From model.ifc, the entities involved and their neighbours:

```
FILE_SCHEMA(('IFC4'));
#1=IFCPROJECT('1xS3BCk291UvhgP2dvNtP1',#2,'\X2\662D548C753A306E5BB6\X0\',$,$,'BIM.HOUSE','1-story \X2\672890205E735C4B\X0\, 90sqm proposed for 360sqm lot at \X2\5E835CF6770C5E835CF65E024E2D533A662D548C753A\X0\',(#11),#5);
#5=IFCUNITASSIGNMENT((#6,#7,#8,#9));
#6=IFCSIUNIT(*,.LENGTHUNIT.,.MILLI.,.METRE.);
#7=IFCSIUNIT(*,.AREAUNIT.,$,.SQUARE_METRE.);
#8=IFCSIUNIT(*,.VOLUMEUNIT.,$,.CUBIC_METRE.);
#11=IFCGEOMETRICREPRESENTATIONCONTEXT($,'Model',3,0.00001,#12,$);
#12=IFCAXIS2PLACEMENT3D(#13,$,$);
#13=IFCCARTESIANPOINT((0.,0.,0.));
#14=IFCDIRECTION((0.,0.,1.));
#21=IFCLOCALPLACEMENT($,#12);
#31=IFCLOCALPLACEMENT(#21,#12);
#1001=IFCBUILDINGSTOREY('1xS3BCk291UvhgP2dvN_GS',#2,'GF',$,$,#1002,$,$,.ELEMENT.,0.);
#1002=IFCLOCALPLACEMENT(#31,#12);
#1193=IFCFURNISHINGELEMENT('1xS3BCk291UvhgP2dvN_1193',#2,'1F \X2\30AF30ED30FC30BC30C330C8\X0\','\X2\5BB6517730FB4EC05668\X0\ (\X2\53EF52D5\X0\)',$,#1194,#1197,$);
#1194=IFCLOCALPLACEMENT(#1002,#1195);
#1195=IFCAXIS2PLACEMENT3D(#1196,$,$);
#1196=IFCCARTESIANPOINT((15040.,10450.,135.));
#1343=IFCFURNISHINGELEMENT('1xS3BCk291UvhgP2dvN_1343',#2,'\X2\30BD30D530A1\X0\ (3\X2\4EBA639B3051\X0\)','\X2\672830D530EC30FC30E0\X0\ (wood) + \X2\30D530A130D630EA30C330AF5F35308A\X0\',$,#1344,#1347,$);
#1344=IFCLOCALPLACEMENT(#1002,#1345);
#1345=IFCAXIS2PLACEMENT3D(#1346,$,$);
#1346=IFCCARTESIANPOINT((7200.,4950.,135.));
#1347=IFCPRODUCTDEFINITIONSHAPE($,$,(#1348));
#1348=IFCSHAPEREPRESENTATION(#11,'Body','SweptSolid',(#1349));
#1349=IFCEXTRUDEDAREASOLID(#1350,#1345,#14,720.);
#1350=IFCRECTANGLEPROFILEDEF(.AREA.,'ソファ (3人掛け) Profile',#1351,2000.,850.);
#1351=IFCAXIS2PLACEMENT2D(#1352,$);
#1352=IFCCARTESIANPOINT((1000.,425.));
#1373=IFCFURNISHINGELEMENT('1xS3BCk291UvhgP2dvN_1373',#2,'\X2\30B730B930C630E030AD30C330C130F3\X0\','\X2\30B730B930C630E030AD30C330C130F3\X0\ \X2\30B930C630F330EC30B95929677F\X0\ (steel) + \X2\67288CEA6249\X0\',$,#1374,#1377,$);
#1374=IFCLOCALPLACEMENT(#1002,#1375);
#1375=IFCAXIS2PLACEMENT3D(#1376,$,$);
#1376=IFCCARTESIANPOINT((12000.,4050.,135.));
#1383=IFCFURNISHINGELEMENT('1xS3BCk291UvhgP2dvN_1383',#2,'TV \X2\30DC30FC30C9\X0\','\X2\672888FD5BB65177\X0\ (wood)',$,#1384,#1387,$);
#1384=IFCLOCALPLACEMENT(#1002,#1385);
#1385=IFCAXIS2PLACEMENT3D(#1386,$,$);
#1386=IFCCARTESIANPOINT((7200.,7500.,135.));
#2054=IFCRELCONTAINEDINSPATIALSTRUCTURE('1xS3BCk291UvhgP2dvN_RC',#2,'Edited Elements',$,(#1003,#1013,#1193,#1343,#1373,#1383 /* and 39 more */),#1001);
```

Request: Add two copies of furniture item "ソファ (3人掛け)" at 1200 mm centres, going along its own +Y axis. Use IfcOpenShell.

```python
import ifcopenshell
import ifcopenshell.api.geometry
import ifcopenshell.api.root
import ifcopenshell.util.element
import ifcopenshell.util.placement

model = ifcopenshell.open("model.ifc")


def reuse_history(source, copy):
    """copy_class also copies each property set's owner history, people and application; keep the originals."""
    for rel in copy.IsDefinedBy:
        if rel.is_a("IfcRelDefinesByProperties") and (history := rel.RelatingPropertyDefinition.OwnerHistory):
            rel.RelatingPropertyDefinition.OwnerHistory = source.OwnerHistory
            ifcopenshell.util.element.remove_deep2(model, history)


source = model.by_id(1343)
base = ifcopenshell.util.placement.get_local_placement(source.ObjectPlacement)
step = base[:3, 1] * 1200.0

for i in range(1, 3):
    copy = ifcopenshell.api.root.copy_class(model, product=source)
    copy.Representation = ifcopenshell.util.element.copy_deep(
        model, source.Representation, exclude=["IfcGeometricRepresentationContext", "IfcRepresentationMap"]
    )
    reuse_history(source, copy)
    matrix = base.copy()
    matrix[:3, 3] += i * step
    print("added at", matrix[:3, 3].round(3) + 0.0)
    ifcopenshell.api.geometry.edit_object_placement(model, product=copy, matrix=matrix, is_si=False)

model.write("model_updated.ifc")
```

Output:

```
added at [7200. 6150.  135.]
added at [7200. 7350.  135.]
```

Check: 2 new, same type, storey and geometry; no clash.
